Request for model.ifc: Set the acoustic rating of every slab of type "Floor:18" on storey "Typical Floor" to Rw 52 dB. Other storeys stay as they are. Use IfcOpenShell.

First a look at what the model holds.

```python
import ifcopenshell
import ifcopenshell.util.element

model = ifcopenshell.open("model.ifc")
print(model.schema)
storey = next(s for s in model.by_type("IfcBuildingStorey") if s.Name == "Typical Floor")
slabs = [e for e in ifcopenshell.util.element.get_decomposition(storey) if e.is_a("IfcSlab")]
seen = {}
for e in slabs:
    element_type = ifcopenshell.util.element.get_type(e)
    key = (element_type.Name if element_type != e and element_type else None, ifcopenshell.util.element.get_pset(e, "Pset_SlabCommon", "AcousticRating"))
    seen[key] = seen.get(key, 0) + 1
for (name, value), count in sorted(seen.items(), key=str):
    print(count, "x", name, "|", value)
```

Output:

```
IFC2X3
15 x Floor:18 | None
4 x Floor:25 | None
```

```python
import ifcopenshell
import ifcopenshell.api.pset
import ifcopenshell.util.element

model = ifcopenshell.open("model.ifc")

storey = next(s for s in model.by_type("IfcBuildingStorey") if s.Name == "Typical Floor")
slabs = [e for e in ifcopenshell.util.element.get_decomposition(storey) if e.is_a("IfcSlab")]

count = 0
for e in slabs:
    element_type = ifcopenshell.util.element.get_type(e)
    if element_type in (None, e) or element_type.Name != "Floor:18":
        continue
    # add_pset returns the element's existing set when there is one.
    pset = ifcopenshell.api.pset.add_pset(model, product=e, name="Pset_SlabCommon")
    ifcopenshell.api.pset.edit_pset(model, pset=pset, properties={"AcousticRating": "Rw 52 dB"})
    count += 1

print(count, "slabs updated")

model.write("model-out.ifc")
```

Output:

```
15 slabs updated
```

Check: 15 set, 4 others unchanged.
